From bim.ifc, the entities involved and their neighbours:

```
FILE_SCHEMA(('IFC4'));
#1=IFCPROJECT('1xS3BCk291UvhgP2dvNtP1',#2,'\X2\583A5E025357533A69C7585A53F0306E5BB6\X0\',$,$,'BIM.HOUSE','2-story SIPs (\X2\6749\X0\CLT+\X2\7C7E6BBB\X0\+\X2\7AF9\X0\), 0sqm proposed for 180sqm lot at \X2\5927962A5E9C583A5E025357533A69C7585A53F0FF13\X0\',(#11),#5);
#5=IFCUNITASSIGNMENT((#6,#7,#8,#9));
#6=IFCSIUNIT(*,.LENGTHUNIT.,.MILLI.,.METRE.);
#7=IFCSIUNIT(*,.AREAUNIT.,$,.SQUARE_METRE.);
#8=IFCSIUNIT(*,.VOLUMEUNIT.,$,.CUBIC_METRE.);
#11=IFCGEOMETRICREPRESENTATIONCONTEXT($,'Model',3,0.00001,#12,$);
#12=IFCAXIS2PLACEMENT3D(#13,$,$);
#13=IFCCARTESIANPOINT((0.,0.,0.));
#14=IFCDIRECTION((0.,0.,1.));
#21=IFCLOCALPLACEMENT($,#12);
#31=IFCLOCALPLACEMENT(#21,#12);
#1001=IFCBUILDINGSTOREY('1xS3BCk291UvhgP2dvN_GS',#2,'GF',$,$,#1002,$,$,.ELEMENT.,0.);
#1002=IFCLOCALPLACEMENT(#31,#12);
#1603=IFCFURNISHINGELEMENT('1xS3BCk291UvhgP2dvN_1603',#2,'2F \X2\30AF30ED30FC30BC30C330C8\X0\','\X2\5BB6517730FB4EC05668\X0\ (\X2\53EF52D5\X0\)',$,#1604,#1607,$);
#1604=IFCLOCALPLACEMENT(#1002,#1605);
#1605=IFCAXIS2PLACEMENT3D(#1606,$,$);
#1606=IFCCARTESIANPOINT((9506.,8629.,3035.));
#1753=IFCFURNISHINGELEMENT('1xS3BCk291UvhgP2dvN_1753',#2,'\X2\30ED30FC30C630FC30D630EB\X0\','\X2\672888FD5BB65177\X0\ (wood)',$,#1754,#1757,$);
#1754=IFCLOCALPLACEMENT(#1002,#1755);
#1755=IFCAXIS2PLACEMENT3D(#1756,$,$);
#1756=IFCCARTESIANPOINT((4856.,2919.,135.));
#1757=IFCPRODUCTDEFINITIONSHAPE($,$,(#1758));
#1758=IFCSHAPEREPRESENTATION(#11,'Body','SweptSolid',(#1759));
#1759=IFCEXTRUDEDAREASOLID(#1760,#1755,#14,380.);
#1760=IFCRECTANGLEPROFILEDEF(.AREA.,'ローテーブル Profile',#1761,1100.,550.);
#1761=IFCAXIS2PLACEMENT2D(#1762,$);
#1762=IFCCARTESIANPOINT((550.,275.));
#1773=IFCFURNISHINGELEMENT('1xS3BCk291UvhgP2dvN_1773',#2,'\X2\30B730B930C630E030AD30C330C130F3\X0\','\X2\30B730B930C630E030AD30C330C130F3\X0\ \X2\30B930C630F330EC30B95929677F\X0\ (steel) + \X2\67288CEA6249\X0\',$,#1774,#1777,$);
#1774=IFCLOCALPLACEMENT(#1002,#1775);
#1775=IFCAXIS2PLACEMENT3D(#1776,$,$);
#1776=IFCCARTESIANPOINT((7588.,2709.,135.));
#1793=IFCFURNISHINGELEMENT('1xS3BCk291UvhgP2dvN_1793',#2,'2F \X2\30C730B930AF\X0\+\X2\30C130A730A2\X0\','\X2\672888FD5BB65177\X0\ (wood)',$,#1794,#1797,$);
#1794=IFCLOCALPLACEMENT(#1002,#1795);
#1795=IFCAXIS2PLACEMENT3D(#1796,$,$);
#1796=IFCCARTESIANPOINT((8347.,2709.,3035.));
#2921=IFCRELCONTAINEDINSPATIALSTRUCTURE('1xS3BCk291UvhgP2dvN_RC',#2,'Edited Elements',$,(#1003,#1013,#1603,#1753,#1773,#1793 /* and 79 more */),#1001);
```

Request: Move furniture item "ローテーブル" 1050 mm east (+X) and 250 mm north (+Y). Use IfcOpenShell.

```python
import ifcopenshell
import ifcopenshell.api.geometry
import ifcopenshell.util.placement
import ifcopenshell.util.unit

model = ifcopenshell.open("bim.ifc")
unit_scale = ifcopenshell.util.unit.calculate_unit_scale(model)

item = model.by_guid("1xS3BCk291UvhgP2dvN_1753")
matrix = ifcopenshell.util.placement.get_local_placement(item.ObjectPlacement)
matrix[0, 3] += 1.05 / unit_scale
matrix[1, 3] += 0.25 / unit_scale
ifcopenshell.api.geometry.edit_object_placement(model, product=item, matrix=matrix, is_si=False)

print(ifcopenshell.util.placement.get_local_placement(item.ObjectPlacement).round(3) + 0.0)

model.write("bim_updated.ifc")
```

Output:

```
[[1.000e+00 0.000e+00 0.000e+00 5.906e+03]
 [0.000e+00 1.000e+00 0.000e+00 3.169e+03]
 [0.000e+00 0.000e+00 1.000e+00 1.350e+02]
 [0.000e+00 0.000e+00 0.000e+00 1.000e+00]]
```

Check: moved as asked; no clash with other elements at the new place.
